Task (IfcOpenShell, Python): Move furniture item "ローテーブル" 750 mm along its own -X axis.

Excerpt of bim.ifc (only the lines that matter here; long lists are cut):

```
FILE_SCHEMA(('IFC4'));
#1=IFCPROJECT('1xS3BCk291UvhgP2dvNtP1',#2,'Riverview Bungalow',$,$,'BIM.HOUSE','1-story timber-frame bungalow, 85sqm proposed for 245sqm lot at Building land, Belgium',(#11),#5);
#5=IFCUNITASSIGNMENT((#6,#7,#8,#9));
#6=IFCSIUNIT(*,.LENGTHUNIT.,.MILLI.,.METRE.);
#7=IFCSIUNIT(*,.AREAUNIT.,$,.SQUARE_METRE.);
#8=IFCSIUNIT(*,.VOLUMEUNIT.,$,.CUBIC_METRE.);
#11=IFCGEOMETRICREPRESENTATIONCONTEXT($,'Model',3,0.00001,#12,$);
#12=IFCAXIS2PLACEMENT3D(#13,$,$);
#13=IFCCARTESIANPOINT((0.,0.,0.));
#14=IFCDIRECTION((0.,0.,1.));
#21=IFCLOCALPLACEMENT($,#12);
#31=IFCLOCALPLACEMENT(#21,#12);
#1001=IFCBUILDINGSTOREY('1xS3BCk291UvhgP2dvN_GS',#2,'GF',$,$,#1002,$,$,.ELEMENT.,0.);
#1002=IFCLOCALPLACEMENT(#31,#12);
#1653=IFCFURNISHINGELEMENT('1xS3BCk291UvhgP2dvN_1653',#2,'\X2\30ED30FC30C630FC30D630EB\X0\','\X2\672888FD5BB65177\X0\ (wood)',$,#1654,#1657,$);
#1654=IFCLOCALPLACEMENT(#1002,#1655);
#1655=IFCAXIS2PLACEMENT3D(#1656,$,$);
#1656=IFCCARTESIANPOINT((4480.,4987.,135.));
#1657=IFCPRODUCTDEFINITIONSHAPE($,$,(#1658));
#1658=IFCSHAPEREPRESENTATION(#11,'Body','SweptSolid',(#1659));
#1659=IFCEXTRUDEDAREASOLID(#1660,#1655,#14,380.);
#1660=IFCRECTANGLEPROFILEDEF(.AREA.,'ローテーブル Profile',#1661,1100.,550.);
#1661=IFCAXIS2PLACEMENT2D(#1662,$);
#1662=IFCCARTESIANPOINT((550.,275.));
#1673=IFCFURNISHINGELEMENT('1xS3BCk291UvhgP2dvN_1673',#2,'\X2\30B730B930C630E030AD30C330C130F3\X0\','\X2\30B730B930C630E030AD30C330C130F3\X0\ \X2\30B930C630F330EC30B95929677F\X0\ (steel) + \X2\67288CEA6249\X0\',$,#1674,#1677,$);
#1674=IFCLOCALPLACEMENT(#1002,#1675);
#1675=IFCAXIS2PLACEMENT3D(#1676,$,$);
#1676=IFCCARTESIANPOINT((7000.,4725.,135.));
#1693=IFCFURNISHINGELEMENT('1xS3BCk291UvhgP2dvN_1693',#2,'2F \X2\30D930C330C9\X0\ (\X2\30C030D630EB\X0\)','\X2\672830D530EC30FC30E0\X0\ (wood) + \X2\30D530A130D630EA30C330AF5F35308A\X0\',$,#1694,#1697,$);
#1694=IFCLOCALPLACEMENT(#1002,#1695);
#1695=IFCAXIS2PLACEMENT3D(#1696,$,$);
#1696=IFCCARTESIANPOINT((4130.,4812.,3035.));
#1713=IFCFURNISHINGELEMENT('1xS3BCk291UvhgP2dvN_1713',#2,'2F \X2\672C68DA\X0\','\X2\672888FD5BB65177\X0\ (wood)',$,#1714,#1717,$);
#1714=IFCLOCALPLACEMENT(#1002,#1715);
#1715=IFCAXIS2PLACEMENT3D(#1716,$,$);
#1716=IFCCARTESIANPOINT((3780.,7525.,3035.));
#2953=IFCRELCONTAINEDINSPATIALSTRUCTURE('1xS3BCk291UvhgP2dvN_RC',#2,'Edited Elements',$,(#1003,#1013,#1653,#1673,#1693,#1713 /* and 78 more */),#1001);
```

```python
import ifcopenshell
import ifcopenshell.api.geometry
import ifcopenshell.util.placement
import ifcopenshell.util.unit

model = ifcopenshell.open("bim.ifc")
unit_scale = ifcopenshell.util.unit.calculate_unit_scale(model)

item = model.by_id(1653)
matrix = ifcopenshell.util.placement.get_local_placement(item.ObjectPlacement)
matrix[:3, 3] -= matrix[:3, 0] * 0.75 / unit_scale
ifcopenshell.api.geometry.edit_object_placement(model, product=item, matrix=matrix, is_si=False)

print(ifcopenshell.util.placement.get_local_placement(item.ObjectPlacement).round(3) + 0.0)

model.write("bim_updated.ifc")
```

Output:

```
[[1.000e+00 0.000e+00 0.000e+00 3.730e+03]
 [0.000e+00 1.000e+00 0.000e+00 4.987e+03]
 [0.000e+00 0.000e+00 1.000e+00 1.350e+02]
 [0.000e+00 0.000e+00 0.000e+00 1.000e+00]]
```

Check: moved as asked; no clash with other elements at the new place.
